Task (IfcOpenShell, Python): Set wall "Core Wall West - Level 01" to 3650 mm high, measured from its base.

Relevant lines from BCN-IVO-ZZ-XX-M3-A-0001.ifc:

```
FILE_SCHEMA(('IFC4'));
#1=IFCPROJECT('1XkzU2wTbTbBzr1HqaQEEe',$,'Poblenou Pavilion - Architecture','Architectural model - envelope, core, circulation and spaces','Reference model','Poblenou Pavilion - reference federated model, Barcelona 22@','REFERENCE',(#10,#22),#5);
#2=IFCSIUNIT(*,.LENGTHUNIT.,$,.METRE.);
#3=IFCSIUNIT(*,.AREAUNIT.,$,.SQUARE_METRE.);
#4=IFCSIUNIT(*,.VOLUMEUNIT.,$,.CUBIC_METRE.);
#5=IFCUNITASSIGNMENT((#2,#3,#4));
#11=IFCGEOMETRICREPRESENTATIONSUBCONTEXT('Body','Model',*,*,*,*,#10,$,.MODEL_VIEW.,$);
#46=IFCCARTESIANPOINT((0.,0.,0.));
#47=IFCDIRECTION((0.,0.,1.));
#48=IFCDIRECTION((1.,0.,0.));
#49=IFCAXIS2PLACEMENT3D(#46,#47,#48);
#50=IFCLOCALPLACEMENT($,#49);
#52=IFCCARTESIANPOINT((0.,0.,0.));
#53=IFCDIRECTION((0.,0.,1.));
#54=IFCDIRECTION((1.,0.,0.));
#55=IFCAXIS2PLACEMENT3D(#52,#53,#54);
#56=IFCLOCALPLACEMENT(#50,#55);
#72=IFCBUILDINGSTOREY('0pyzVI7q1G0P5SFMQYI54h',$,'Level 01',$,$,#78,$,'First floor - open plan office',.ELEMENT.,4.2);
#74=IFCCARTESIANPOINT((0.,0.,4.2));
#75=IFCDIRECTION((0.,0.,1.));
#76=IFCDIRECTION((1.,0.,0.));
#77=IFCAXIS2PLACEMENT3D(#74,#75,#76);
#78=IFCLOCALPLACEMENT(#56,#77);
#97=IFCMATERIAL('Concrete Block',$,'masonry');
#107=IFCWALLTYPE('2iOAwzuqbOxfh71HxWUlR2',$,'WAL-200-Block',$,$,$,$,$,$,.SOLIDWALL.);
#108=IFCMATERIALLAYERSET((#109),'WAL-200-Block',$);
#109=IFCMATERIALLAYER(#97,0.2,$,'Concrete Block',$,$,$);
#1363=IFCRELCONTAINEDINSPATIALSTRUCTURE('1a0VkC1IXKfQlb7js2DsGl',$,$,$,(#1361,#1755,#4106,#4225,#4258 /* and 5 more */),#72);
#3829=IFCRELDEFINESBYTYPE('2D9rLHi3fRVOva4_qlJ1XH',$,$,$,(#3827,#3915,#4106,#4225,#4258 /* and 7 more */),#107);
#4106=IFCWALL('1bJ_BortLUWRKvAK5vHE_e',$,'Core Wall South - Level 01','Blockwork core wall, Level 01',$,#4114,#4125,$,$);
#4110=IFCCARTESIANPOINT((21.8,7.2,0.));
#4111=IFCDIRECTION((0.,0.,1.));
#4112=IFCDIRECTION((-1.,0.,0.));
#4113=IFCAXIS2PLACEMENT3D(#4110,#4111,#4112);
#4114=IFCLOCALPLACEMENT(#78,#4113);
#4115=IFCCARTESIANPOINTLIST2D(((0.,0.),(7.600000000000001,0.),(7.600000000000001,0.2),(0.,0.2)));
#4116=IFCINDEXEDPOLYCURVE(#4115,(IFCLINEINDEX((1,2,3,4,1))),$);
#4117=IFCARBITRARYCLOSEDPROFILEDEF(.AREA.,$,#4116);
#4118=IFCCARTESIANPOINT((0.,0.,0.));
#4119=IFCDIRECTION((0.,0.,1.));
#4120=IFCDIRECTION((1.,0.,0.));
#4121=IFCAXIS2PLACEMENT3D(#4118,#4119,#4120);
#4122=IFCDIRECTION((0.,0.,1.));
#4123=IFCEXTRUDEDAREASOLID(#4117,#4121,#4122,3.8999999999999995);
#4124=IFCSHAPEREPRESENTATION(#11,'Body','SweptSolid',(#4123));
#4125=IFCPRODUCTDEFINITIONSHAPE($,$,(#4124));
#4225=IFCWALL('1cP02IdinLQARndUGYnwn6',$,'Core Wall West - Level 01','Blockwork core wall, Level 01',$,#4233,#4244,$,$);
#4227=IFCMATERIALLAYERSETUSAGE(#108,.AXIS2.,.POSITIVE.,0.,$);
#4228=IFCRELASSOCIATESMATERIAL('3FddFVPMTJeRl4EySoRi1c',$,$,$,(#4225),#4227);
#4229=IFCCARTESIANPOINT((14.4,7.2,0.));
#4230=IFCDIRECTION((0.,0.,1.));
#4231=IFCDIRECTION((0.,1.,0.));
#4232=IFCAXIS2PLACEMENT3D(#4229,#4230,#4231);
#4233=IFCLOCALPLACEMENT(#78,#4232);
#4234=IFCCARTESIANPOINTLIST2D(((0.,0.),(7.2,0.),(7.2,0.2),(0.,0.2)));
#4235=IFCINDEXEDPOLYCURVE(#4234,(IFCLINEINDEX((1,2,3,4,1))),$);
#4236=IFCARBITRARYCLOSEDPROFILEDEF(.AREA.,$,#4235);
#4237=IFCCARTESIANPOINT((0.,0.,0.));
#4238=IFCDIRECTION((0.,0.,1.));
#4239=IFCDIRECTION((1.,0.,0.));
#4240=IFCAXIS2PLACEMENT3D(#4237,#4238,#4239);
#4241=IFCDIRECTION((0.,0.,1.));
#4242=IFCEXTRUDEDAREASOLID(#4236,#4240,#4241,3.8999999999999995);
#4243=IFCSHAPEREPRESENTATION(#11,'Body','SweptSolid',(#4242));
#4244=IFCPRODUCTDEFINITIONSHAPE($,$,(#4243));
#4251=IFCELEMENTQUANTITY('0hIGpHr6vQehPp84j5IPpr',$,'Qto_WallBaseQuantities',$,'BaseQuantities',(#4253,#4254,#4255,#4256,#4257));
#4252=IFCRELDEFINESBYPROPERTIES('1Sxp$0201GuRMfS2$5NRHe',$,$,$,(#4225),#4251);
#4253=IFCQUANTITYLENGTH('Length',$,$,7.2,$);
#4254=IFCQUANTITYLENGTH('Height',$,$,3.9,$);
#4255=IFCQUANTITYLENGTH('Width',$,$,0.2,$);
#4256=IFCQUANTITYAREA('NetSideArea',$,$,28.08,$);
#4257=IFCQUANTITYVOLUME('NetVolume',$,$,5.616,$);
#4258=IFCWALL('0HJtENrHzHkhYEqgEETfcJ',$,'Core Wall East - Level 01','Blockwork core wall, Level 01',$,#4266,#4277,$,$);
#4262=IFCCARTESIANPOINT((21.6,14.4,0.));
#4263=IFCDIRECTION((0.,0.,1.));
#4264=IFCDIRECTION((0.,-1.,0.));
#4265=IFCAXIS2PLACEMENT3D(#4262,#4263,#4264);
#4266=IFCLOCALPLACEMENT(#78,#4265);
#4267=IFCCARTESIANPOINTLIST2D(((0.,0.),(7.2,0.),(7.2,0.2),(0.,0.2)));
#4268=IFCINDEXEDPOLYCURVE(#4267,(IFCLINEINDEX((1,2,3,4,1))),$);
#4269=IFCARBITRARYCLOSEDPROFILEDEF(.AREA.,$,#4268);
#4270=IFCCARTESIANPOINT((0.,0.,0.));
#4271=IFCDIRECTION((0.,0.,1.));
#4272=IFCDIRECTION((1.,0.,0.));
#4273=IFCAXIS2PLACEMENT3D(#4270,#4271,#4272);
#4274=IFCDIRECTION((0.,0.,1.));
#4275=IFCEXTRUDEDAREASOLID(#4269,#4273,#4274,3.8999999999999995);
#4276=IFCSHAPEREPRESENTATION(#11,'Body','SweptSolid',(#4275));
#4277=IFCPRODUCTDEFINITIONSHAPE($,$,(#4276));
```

```python
import ifcopenshell
import ifcopenshell.api.pset
import ifcopenshell.geom
import ifcopenshell.util.element
import ifcopenshell.util.representation
import ifcopenshell.util.shape
import ifcopenshell.util.unit

model = ifcopenshell.open("BCN-IVO-ZZ-XX-M3-A-0001.ifc")
unit_scale = ifcopenshell.util.unit.calculate_unit_scale(model)
area_scale = ifcopenshell.util.unit.calculate_unit_scale(model, "AREAUNIT")
volume_scale = ifcopenshell.util.unit.calculate_unit_scale(model, "VOLUMEUNIT")
settings = ifcopenshell.geom.settings()


def volume(element):
    """Net volume in cubic metres, openings subtracted."""
    shape = ifcopenshell.geom.create_shape(settings, element)
    return ifcopenshell.util.shape.get_volume(shape.geometry)


wall = model.by_id(4225)
before = volume(wall)

body = ifcopenshell.util.representation.get_representation(wall, "Model", "Body")
solid = body.Items[0]
old_height = solid.Depth
solid.Depth = 3.65 / unit_scale
after = volume(wall)
thickness = 0.2  # wall thickness in metres

# Update the stored height, areas and volumes.
qto = model.by_id(ifcopenshell.util.element.get_pset(wall, "Qto_WallBaseQuantities", should_inherit=False)["id"])
ifcopenshell.api.pset.edit_qto(model, qto=qto, properties={
    "Height": solid.Depth,
    "NetSideArea": after / thickness / area_scale,
    "NetVolume": after / volume_scale,
})

print(f"height {old_height:g} -> {solid.Depth:g}, volume {before:.3f} -> {after:.3f} m3")

model.write("BCN-IVO-ZZ-XX-M3-A-0001_v2.ifc")
```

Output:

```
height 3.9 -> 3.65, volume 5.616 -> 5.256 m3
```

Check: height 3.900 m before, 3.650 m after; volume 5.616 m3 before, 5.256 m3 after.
